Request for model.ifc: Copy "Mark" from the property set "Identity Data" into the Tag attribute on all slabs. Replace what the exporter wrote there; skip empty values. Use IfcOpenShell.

First a look at what the model holds.

```python
import ifcopenshell
import ifcopenshell.util.element

model = ifcopenshell.open("model.ifc")
print(model.schema)
slabs = model.by_type("IfcSlab")
print(len(slabs), "slabs")
for e in slabs[:8]:
    source = ifcopenshell.util.element.get_pset(e, "Identity Data", "Mark")
    target = e.Tag
    print(e.id(), repr(source), repr(target), sep=" | ")
```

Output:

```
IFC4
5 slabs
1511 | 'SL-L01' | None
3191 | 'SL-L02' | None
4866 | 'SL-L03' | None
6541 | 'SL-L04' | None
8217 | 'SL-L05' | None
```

```python
import ifcopenshell
import ifcopenshell.util.element

model = ifcopenshell.open("model.ifc")

count = 0
for e in model.by_type("IfcSlab"):
    value = ifcopenshell.util.element.get_pset(e, "Identity Data", "Mark")
    current = e.Tag
    if not value or not value.strip() or current == value:
        continue
    e.Tag = value
    count += 1

print(count, "slabs updated")

model.write("model_rev.ifc")
```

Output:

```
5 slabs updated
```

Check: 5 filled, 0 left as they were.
